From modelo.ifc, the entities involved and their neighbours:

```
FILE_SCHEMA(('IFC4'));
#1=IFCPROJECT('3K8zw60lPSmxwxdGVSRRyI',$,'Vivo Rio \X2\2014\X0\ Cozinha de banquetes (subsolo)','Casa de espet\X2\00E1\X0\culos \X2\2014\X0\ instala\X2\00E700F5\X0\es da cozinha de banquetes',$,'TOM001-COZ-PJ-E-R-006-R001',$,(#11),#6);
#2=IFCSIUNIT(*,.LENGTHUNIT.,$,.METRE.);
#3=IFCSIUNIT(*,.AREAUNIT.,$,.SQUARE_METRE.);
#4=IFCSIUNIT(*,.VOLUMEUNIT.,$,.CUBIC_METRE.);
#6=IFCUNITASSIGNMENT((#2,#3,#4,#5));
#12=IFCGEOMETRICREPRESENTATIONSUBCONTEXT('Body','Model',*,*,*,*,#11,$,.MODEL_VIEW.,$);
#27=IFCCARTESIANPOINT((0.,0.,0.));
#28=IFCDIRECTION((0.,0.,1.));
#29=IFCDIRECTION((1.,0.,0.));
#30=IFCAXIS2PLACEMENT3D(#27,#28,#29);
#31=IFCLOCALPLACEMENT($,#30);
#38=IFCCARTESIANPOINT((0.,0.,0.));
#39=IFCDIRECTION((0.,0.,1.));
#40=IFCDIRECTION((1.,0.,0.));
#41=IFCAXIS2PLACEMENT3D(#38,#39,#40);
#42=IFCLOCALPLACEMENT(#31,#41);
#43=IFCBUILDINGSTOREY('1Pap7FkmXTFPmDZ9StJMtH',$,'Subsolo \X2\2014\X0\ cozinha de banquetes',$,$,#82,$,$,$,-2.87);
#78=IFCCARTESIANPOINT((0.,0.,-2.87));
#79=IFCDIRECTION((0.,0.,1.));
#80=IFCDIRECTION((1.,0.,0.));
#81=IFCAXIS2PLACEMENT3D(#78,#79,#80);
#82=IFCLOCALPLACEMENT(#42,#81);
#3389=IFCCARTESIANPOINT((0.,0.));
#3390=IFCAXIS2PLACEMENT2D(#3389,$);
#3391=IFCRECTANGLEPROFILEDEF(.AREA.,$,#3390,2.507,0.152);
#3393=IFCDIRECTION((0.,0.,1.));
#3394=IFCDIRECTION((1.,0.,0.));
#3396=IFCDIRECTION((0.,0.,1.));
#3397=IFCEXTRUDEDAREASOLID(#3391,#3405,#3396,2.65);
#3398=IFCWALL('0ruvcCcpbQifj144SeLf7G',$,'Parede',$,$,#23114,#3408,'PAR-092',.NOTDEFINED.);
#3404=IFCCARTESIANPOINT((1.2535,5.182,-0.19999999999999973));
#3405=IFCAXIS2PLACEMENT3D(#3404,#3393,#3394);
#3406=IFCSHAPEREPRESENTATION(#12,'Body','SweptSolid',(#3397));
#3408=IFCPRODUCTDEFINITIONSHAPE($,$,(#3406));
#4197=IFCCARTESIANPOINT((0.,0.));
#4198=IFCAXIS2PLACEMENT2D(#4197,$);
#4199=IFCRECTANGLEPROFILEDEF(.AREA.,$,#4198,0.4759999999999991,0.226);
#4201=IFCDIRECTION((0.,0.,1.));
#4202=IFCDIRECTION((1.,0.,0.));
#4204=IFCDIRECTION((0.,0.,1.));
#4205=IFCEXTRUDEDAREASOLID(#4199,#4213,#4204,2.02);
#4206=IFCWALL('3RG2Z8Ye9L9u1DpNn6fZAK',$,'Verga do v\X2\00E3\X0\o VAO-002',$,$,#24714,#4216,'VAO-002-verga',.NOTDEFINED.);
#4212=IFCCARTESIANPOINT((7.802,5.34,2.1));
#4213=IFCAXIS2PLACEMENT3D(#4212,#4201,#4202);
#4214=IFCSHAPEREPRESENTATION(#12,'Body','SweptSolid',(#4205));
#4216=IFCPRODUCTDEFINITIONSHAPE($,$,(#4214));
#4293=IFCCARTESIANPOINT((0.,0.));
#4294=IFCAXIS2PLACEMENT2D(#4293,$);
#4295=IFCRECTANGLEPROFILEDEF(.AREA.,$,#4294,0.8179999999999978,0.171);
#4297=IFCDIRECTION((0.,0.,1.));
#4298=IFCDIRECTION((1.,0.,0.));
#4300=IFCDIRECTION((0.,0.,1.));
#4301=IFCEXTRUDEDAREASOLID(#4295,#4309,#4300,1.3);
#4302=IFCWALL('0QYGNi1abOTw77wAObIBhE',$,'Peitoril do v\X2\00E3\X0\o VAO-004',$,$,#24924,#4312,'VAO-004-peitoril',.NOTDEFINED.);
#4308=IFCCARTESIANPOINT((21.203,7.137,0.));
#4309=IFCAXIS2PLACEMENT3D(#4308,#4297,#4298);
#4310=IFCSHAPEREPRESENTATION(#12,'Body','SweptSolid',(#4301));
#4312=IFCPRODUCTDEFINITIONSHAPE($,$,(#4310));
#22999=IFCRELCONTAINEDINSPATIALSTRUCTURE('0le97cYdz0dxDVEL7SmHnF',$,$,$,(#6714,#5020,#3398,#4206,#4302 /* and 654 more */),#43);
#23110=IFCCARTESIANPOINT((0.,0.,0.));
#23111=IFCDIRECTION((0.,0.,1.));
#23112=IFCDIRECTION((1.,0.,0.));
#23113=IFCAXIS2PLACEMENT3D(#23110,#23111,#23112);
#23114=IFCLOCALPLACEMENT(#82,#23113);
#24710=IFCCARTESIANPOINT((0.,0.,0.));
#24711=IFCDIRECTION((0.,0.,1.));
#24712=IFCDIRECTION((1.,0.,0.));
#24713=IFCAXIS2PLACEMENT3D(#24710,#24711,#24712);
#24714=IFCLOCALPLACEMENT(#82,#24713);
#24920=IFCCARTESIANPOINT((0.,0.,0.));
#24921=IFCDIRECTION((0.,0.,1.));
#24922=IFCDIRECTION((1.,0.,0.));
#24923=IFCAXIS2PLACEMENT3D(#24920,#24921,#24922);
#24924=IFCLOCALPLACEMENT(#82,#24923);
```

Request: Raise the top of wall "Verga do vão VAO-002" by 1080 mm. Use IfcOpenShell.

```python
import ifcopenshell
import ifcopenshell.geom
import ifcopenshell.util.representation
import ifcopenshell.util.shape
import ifcopenshell.util.unit

model = ifcopenshell.open("modelo.ifc")
unit_scale = ifcopenshell.util.unit.calculate_unit_scale(model)
settings = ifcopenshell.geom.settings()


def volume(element):
    """Net volume in cubic metres, openings subtracted."""
    shape = ifcopenshell.geom.create_shape(settings, element)
    return ifcopenshell.util.shape.get_volume(shape.geometry)


wall = model.by_guid("3RG2Z8Ye9L9u1DpNn6fZAK")
before = volume(wall)

body = ifcopenshell.util.representation.get_representation(wall, "Model", "Body")
solid = body.Items[0]
old_height = solid.Depth
solid.Depth += 1.08 / unit_scale
after = volume(wall)

print(f"height {old_height:g} -> {solid.Depth:g}, volume {before:.3f} -> {after:.3f} m3")

model.write("modelo_v2.ifc")
```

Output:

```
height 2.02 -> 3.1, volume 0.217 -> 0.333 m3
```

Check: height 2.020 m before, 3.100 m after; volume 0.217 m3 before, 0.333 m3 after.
